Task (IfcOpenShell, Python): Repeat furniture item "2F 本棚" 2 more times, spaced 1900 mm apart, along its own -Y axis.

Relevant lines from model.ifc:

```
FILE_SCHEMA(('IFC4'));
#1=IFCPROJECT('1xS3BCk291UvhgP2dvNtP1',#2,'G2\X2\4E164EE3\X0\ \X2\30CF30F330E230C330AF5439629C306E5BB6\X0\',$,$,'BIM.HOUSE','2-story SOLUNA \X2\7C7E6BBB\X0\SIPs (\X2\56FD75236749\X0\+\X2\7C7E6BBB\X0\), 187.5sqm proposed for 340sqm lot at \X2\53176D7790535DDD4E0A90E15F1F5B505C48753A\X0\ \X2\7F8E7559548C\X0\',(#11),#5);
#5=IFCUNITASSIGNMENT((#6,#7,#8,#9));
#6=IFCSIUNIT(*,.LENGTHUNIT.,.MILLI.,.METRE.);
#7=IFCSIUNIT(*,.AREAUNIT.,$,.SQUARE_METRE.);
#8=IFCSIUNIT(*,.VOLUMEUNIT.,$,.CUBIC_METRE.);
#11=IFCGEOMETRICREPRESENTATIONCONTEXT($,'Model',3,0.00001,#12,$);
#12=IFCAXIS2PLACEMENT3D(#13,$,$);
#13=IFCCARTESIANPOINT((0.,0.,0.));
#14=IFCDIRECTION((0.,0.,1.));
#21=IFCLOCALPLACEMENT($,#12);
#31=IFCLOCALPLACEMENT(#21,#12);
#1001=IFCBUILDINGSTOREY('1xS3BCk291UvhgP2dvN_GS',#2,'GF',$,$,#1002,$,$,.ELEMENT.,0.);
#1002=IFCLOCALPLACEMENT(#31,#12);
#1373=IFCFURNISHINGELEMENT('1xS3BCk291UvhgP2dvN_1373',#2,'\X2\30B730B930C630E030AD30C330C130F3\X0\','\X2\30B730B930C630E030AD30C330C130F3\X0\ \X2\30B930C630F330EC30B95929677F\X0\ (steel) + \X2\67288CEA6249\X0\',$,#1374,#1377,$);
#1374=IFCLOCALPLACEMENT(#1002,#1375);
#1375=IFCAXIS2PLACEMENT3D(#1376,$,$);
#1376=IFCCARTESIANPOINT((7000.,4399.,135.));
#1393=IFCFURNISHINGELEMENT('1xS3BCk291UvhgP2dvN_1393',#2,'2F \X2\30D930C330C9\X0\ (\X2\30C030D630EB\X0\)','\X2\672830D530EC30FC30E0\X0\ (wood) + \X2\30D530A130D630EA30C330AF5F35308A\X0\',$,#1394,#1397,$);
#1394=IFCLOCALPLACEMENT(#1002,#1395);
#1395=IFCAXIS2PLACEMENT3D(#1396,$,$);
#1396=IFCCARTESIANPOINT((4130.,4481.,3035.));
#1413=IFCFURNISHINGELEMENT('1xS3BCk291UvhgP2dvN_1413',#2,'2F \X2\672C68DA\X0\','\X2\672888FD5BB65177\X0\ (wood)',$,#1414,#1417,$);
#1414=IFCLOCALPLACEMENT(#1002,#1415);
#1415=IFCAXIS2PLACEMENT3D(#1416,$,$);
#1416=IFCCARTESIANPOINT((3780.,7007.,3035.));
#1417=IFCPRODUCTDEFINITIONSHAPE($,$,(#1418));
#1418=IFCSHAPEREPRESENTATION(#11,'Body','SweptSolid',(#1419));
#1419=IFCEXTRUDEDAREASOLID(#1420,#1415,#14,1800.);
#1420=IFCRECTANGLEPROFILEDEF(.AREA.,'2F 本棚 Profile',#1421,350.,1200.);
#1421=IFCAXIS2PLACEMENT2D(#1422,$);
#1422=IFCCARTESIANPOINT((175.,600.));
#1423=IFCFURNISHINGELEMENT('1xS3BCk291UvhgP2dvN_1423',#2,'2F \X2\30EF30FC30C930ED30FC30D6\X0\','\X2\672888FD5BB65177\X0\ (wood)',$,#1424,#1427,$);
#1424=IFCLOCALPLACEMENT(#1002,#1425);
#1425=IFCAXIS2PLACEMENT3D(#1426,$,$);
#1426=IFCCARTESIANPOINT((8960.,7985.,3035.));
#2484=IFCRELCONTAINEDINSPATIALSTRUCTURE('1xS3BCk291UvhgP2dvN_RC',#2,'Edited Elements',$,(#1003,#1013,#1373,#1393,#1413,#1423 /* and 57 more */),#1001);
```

```python
import ifcopenshell
import ifcopenshell.api.geometry
import ifcopenshell.api.root
import ifcopenshell.util.element
import ifcopenshell.util.placement

model = ifcopenshell.open("model.ifc")


def reuse_history(source, copy):
    """copy_class also copies each property set's owner history, people and application; keep the originals."""
    for rel in copy.IsDefinedBy:
        if rel.is_a("IfcRelDefinesByProperties") and (history := rel.RelatingPropertyDefinition.OwnerHistory):
            rel.RelatingPropertyDefinition.OwnerHistory = source.OwnerHistory
            ifcopenshell.util.element.remove_deep2(model, history)


source = model.by_guid("1xS3BCk291UvhgP2dvN_1413")
base = ifcopenshell.util.placement.get_local_placement(source.ObjectPlacement)
step = -base[:3, 1] * 1900.0

for i in range(1, 3):
    copy = ifcopenshell.api.root.copy_class(model, product=source)
    copy.Representation = ifcopenshell.util.element.copy_deep(
        model, source.Representation, exclude=["IfcGeometricRepresentationContext", "IfcRepresentationMap"]
    )
    reuse_history(source, copy)
    matrix = base.copy()
    matrix[:3, 3] += i * step
    print("added at", matrix[:3, 3].round(3) + 0.0)
    ifcopenshell.api.geometry.edit_object_placement(model, product=copy, matrix=matrix, is_si=False)

model.write("model_rev.ifc")
```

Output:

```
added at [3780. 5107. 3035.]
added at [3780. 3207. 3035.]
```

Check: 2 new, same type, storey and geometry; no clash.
